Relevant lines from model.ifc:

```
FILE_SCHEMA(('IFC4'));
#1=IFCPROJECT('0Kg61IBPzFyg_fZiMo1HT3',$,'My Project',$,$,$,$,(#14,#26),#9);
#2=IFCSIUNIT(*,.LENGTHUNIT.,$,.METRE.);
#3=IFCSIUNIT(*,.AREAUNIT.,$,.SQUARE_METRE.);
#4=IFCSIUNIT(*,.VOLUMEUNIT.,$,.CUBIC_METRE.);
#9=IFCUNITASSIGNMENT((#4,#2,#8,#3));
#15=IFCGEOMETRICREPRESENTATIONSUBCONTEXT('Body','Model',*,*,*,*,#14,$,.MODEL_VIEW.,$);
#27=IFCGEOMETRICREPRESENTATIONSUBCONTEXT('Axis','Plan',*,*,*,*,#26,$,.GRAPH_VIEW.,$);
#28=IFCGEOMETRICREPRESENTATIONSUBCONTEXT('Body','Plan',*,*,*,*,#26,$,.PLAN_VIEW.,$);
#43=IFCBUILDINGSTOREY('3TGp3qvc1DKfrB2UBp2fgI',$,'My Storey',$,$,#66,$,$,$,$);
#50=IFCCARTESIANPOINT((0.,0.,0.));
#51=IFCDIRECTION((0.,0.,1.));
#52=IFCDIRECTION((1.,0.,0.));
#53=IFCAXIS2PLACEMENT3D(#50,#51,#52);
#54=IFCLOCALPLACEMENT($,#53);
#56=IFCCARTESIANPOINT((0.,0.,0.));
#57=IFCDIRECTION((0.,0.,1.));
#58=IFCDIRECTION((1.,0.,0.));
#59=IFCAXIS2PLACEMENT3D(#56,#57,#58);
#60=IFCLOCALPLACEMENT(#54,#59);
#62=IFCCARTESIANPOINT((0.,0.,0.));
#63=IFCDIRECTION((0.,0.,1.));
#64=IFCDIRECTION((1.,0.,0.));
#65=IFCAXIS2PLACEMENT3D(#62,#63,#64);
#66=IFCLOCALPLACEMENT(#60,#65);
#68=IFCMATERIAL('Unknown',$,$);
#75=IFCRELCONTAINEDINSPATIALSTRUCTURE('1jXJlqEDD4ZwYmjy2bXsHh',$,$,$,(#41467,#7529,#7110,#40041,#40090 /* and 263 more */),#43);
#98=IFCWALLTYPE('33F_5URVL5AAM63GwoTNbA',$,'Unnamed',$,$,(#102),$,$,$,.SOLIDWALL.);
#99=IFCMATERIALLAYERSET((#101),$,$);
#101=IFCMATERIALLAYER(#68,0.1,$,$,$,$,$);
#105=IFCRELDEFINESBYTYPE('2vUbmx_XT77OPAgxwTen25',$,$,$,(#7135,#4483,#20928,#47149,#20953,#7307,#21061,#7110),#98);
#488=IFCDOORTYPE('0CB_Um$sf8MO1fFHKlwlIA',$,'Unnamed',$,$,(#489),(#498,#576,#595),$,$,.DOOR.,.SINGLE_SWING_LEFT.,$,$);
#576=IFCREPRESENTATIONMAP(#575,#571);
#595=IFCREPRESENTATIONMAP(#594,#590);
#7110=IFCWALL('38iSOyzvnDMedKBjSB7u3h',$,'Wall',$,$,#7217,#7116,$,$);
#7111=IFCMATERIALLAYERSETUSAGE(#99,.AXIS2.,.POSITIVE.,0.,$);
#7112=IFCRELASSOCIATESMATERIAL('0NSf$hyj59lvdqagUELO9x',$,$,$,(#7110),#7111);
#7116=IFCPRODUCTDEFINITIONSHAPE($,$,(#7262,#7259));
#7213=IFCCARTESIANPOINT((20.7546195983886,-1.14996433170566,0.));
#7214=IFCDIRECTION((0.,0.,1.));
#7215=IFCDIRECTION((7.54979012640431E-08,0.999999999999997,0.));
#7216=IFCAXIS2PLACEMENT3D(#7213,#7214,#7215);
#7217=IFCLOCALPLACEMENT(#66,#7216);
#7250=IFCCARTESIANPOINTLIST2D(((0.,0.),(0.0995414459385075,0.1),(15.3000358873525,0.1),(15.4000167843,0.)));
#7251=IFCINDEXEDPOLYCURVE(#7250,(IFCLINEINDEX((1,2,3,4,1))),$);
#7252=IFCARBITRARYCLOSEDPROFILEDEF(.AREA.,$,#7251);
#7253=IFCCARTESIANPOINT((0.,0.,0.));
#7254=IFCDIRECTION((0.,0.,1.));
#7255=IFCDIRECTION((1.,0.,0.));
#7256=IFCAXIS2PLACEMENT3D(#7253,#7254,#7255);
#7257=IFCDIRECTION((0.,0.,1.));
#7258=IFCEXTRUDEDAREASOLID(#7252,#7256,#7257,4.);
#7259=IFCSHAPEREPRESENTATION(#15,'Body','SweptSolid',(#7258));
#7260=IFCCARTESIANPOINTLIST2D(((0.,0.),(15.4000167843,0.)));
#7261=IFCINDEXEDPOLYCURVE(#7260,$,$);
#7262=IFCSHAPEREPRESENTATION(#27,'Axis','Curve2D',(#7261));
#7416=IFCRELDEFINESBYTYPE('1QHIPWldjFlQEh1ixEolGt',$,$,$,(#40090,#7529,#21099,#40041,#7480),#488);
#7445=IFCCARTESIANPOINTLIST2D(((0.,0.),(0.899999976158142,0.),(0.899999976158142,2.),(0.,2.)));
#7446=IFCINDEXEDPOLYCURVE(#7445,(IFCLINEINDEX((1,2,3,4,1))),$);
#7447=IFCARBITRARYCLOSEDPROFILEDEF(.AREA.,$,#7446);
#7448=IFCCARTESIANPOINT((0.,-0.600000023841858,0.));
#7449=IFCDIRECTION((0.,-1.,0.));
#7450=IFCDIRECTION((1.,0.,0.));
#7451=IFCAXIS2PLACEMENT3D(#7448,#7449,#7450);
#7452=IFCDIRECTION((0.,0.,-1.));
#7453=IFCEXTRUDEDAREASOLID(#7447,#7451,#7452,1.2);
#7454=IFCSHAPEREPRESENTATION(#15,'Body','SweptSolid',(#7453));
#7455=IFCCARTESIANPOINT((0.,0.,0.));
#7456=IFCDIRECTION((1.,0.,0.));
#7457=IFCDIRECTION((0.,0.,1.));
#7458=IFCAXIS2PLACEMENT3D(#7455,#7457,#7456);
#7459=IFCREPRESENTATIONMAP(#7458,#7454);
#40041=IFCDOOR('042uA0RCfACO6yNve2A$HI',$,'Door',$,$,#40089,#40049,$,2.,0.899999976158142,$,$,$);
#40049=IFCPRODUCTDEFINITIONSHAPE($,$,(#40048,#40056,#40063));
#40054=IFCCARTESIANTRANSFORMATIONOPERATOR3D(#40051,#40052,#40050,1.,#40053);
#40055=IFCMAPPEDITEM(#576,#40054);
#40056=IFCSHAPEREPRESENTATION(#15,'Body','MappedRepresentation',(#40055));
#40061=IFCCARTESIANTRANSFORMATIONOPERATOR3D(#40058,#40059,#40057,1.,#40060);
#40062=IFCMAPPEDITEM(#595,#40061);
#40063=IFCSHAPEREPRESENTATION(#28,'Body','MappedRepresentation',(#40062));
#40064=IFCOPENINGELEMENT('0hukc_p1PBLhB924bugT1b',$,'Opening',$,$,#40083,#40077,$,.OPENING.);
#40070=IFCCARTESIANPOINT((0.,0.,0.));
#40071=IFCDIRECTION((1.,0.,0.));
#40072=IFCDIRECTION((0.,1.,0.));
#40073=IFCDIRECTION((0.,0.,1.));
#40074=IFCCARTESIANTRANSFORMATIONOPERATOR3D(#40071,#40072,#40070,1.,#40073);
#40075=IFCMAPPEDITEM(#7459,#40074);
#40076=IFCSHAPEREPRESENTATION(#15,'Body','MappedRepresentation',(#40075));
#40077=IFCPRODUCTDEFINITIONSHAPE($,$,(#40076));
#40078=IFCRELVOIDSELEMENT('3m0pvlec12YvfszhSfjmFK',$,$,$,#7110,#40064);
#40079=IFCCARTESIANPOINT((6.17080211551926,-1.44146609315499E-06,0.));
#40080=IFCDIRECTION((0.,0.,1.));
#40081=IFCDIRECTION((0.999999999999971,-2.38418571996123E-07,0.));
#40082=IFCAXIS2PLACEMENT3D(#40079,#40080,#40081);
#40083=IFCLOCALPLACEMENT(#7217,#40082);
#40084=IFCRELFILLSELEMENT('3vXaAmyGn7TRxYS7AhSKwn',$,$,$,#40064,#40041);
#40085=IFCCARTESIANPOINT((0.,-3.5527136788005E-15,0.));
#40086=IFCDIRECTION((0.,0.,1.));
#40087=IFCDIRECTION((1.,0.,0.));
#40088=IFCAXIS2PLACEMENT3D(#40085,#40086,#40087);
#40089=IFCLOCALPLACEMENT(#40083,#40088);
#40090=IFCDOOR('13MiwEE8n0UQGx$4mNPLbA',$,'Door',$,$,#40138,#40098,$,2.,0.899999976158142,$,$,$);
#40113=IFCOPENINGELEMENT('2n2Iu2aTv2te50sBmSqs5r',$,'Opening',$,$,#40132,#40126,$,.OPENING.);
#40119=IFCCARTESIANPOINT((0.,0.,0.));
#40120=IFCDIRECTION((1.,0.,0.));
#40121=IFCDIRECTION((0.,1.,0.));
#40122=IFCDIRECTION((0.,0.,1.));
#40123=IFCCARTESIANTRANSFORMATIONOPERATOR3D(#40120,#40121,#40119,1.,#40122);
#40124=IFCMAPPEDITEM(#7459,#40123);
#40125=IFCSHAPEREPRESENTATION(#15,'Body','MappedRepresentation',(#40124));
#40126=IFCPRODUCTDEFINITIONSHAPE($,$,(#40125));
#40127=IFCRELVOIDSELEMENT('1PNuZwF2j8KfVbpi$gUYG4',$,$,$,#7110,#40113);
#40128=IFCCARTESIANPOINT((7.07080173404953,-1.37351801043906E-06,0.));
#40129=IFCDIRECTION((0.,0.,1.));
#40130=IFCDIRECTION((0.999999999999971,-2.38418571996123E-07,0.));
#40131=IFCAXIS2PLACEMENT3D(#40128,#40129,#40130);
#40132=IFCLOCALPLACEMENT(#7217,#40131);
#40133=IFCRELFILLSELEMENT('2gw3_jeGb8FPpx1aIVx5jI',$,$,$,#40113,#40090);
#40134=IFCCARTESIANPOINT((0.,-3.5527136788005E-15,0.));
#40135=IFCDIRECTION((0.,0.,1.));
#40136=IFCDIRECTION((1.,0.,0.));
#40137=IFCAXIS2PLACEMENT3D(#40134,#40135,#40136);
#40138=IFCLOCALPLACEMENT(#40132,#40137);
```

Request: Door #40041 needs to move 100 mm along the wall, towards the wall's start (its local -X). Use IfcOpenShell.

```python
import ifcopenshell
import ifcopenshell.api.geometry
import ifcopenshell.util.placement

model = ifcopenshell.open("model.ifc")

door = model.by_id(40041)
opening = door.FillsVoids[0].RelatingOpeningElement
wall = opening.VoidsElements[0].RelatingBuildingElement

wall_matrix = ifcopenshell.util.placement.get_local_placement(wall.ObjectPlacement)
shift = wall_matrix[:3, 0] * -0.1
before = ifcopenshell.util.placement.get_local_placement(door.ObjectPlacement)[:3, 3].copy()

# The door is placed relative to its opening, so it follows when the opening moves.
matrix = ifcopenshell.util.placement.get_local_placement(opening.ObjectPlacement)
matrix[:3, 3] += shift
ifcopenshell.api.geometry.edit_object_placement(
    model, product=opening, matrix=matrix, is_si=False, should_transform_children=True
)

after = ifcopenshell.util.placement.get_local_placement(door.ObjectPlacement)[:3, 3]
print("door moved by", (after - before).round(3) + 0.0)

model.write("model_v2.ifc")
```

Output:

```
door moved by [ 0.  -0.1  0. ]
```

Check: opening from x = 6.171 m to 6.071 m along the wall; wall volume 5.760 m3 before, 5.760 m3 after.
